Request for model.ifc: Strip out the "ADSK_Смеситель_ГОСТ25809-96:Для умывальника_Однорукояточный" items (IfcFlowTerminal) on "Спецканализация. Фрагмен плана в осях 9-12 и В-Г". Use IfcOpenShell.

First a look at what the model holds.

```python
import ifcopenshell
import ifcopenshell.util.element

model = ifcopenshell.open("model.ifc")
print(model.schema)
storey = next(s for s in model.by_type("IfcBuildingStorey") if s.Name == "Спецканализация. Фрагмен плана в осях 9-12 и В-Г")
terminals = [e for e in ifcopenshell.util.element.get_decomposition(storey) if e.is_a("IfcFlowTerminal")]
seen = {}
for e in terminals:
    element_type = ifcopenshell.util.element.get_type(e)
    name = element_type.Name if element_type not in (None, e) else None
    seen[name] = seen.get(name, 0) + 1
for name, count in sorted(seen.items(), key=str):
    print(count, "x", name)
```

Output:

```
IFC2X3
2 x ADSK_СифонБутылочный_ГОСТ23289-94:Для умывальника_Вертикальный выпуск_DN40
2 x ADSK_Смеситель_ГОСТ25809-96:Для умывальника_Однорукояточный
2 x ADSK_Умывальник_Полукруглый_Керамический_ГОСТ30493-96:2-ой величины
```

```python
import ifcopenshell
import ifcopenshell.api.root
import ifcopenshell.util.element

model = ifcopenshell.open("model.ifc")

storey = next(s for s in model.by_type("IfcBuildingStorey") if s.Name == "Спецканализация. Фрагмен плана в осях 9-12 и В-Г")
terminals = [e for e in ifcopenshell.util.element.get_decomposition(storey) if e.is_a("IfcFlowTerminal")]
targets = [e for e in terminals if (t := ifcopenshell.util.element.get_type(e)) not in (None, e) and t.Name == "ADSK_Смеситель_ГОСТ25809-96:Для умывальника_Однорукояточный"]

for e in targets:
    ifcopenshell.api.root.remove_product(model, product=e)
print(len(targets), "removed")

model.write("model-out.ifc")
```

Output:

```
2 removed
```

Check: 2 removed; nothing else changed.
